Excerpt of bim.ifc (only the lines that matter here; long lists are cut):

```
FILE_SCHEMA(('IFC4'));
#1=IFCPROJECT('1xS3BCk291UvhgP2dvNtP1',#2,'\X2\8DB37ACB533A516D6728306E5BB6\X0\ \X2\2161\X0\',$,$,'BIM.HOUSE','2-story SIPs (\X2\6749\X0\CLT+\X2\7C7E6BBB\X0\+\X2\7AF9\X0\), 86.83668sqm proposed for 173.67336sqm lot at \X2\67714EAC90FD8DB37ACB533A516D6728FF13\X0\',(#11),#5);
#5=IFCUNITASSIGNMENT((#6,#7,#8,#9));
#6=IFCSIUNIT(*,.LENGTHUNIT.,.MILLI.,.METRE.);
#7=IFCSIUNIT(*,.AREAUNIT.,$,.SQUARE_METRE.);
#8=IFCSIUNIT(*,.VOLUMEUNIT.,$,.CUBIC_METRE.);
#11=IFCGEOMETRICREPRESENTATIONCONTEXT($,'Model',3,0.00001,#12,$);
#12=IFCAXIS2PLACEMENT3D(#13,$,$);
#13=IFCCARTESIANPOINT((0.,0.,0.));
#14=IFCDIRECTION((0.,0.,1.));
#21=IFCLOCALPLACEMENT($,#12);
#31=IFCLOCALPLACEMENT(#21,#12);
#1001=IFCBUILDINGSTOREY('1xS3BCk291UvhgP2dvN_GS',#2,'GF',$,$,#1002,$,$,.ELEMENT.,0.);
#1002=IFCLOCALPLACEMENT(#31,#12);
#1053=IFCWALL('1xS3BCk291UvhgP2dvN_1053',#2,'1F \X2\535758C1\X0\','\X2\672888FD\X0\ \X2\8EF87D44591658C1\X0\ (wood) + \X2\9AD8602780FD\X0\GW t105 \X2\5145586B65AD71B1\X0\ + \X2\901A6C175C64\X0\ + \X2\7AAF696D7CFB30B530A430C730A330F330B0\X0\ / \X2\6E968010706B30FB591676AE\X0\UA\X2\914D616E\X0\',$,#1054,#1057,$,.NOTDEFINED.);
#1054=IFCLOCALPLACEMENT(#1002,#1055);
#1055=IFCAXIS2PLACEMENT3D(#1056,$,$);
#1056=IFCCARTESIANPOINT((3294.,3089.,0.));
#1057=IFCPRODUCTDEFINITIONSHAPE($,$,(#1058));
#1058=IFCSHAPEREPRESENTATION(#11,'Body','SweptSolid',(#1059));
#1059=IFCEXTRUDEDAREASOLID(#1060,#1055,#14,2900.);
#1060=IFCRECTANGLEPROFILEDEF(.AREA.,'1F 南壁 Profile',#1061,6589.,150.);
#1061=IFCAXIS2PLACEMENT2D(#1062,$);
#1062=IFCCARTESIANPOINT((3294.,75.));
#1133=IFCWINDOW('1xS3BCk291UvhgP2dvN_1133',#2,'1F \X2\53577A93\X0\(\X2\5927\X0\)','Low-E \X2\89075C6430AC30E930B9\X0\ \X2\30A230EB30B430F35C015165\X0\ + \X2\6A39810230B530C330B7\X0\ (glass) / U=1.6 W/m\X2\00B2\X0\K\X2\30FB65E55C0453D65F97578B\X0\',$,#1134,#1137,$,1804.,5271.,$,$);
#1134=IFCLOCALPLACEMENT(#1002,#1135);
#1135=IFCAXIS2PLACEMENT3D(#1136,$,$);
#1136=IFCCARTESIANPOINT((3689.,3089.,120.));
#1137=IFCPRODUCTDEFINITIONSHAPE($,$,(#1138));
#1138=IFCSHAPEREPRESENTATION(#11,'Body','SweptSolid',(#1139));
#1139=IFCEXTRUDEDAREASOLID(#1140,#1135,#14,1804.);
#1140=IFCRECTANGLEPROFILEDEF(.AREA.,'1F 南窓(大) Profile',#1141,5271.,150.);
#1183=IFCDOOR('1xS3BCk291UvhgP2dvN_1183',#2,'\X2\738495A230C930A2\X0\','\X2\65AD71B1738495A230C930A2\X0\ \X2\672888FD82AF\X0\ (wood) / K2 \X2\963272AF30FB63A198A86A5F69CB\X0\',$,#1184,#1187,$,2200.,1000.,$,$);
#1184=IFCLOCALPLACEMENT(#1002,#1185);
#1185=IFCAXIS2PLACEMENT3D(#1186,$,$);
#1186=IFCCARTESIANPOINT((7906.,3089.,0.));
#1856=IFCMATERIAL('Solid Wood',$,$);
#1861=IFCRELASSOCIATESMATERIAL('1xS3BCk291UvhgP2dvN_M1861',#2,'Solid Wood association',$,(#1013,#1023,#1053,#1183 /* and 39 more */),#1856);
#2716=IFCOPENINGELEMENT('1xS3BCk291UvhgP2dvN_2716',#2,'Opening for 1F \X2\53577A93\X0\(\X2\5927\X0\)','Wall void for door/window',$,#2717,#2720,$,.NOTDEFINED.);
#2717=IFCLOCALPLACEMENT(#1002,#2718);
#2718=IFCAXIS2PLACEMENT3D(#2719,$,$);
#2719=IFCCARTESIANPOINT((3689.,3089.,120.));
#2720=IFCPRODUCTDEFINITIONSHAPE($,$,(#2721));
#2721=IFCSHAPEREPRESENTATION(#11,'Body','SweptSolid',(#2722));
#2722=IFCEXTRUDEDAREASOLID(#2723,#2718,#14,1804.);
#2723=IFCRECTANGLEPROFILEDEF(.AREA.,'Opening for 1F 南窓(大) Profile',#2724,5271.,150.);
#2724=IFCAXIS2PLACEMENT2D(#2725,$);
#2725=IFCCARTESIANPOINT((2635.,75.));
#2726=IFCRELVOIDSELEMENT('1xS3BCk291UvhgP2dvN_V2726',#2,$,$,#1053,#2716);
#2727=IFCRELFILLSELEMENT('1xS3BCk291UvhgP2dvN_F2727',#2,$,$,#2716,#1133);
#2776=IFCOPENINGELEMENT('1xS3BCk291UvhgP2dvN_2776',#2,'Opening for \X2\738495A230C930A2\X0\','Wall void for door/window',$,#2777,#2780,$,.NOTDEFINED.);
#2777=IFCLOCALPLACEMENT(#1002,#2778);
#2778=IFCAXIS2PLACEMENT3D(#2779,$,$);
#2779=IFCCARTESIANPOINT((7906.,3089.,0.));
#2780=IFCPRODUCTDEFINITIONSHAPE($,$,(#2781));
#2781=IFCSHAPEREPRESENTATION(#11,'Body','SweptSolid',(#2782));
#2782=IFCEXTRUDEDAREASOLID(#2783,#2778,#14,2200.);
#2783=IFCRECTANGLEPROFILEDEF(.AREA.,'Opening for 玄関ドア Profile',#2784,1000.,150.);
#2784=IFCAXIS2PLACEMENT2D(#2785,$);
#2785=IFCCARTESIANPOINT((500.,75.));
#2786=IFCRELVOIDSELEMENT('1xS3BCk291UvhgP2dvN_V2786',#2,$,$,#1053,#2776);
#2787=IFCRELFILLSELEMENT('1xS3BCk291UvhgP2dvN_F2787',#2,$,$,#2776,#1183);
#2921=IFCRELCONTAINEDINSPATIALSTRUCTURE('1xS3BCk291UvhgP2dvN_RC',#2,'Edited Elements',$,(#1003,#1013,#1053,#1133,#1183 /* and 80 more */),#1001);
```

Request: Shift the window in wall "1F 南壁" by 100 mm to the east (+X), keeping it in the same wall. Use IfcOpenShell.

```python
import ifcopenshell
import ifcopenshell.api.geometry
import ifcopenshell.util.placement
import ifcopenshell.util.unit

model = ifcopenshell.open("bim.ifc")
unit_scale = ifcopenshell.util.unit.calculate_unit_scale(model)

window = model.by_id(1133)
opening = window.FillsVoids[0].RelatingOpeningElement
wall = opening.VoidsElements[0].RelatingBuildingElement

wall_matrix = ifcopenshell.util.placement.get_local_placement(wall.ObjectPlacement)
shift = wall_matrix[:3, 0] * 0.1 / unit_scale
before = ifcopenshell.util.placement.get_local_placement(window.ObjectPlacement)[:3, 3].copy()

# The window is not placed relative to its opening, so move both.
for product in (opening, window):
    matrix = ifcopenshell.util.placement.get_local_placement(product.ObjectPlacement)
    matrix[:3, 3] += shift
    ifcopenshell.api.geometry.edit_object_placement(model, product=product, matrix=matrix, is_si=False)

after = ifcopenshell.util.placement.get_local_placement(window.ObjectPlacement)[:3, 3]
print("window moved by", (after - before).round(3) + 0.0)

model.write("bim-out.ifc")
```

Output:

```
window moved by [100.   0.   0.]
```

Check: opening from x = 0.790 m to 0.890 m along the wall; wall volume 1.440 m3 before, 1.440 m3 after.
